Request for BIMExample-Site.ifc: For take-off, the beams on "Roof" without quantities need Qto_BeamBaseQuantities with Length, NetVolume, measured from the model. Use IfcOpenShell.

First a look at what the model holds.

```python
import ifcopenshell
import ifcopenshell.util.element
import ifcopenshell.util.unit

model = ifcopenshell.open("BIMExample-Site.ifc")
print(model.schema)
for unit_type in ("LENGTHUNIT", "AREAUNIT", "VOLUMEUNIT"):
    print(unit_type, ifcopenshell.util.unit.calculate_unit_scale(model, unit_type))
storey = next(s for s in model.by_type("IfcBuildingStorey") if s.Name == "Roof")
beams = [e for e in ifcopenshell.util.element.get_decomposition(storey) if e.is_a("IfcBeam")]
for e in sorted(beams, key=lambda e: e.id()):
    print(e.id(), e.is_a(), e.Name, list(ifcopenshell.util.element.get_psets(e, qtos_only=True)), sep=" | ")
```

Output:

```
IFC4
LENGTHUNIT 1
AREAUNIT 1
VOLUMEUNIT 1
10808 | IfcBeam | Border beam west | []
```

```python
import ifcopenshell
import ifcopenshell.api.pset
import ifcopenshell.geom
import ifcopenshell.util.element
import ifcopenshell.util.shape
import ifcopenshell.util.unit

model = ifcopenshell.open("BIMExample-Site.ifc")
unit_scale = ifcopenshell.util.unit.calculate_unit_scale(model)
volume_scale = ifcopenshell.util.unit.calculate_unit_scale(model, "VOLUMEUNIT")
settings = ifcopenshell.geom.settings()

storey = next(s for s in model.by_type("IfcBuildingStorey") if s.Name == "Roof")
beams = [e for e in ifcopenshell.util.element.get_decomposition(storey) if e.is_a("IfcBeam")]

for e in sorted(beams, key=lambda e: e.id()):
    if ifcopenshell.util.element.get_psets(e, qtos_only=True, should_inherit=False):
        continue
    # Geometry comes back in metres, in the element's own axes.
    shape = ifcopenshell.geom.create_shape(settings, e)
    values = {
        "Length": ifcopenshell.util.shape.get_max_xyz(shape.geometry) / unit_scale,
        "NetVolume": ifcopenshell.util.shape.get_volume(shape.geometry) / volume_scale,
    }
    qto = ifcopenshell.api.pset.add_qto(model, product=e, name="Qto_BeamBaseQuantities")
    ifcopenshell.api.pset.edit_qto(model, qto=qto, properties=values)
    print(e.id(), {k: round(v, 3) for k, v in values.items()})

model.write("BIMExample-Site_edited.ifc")
```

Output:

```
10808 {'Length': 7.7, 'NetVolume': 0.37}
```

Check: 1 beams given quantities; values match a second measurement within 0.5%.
